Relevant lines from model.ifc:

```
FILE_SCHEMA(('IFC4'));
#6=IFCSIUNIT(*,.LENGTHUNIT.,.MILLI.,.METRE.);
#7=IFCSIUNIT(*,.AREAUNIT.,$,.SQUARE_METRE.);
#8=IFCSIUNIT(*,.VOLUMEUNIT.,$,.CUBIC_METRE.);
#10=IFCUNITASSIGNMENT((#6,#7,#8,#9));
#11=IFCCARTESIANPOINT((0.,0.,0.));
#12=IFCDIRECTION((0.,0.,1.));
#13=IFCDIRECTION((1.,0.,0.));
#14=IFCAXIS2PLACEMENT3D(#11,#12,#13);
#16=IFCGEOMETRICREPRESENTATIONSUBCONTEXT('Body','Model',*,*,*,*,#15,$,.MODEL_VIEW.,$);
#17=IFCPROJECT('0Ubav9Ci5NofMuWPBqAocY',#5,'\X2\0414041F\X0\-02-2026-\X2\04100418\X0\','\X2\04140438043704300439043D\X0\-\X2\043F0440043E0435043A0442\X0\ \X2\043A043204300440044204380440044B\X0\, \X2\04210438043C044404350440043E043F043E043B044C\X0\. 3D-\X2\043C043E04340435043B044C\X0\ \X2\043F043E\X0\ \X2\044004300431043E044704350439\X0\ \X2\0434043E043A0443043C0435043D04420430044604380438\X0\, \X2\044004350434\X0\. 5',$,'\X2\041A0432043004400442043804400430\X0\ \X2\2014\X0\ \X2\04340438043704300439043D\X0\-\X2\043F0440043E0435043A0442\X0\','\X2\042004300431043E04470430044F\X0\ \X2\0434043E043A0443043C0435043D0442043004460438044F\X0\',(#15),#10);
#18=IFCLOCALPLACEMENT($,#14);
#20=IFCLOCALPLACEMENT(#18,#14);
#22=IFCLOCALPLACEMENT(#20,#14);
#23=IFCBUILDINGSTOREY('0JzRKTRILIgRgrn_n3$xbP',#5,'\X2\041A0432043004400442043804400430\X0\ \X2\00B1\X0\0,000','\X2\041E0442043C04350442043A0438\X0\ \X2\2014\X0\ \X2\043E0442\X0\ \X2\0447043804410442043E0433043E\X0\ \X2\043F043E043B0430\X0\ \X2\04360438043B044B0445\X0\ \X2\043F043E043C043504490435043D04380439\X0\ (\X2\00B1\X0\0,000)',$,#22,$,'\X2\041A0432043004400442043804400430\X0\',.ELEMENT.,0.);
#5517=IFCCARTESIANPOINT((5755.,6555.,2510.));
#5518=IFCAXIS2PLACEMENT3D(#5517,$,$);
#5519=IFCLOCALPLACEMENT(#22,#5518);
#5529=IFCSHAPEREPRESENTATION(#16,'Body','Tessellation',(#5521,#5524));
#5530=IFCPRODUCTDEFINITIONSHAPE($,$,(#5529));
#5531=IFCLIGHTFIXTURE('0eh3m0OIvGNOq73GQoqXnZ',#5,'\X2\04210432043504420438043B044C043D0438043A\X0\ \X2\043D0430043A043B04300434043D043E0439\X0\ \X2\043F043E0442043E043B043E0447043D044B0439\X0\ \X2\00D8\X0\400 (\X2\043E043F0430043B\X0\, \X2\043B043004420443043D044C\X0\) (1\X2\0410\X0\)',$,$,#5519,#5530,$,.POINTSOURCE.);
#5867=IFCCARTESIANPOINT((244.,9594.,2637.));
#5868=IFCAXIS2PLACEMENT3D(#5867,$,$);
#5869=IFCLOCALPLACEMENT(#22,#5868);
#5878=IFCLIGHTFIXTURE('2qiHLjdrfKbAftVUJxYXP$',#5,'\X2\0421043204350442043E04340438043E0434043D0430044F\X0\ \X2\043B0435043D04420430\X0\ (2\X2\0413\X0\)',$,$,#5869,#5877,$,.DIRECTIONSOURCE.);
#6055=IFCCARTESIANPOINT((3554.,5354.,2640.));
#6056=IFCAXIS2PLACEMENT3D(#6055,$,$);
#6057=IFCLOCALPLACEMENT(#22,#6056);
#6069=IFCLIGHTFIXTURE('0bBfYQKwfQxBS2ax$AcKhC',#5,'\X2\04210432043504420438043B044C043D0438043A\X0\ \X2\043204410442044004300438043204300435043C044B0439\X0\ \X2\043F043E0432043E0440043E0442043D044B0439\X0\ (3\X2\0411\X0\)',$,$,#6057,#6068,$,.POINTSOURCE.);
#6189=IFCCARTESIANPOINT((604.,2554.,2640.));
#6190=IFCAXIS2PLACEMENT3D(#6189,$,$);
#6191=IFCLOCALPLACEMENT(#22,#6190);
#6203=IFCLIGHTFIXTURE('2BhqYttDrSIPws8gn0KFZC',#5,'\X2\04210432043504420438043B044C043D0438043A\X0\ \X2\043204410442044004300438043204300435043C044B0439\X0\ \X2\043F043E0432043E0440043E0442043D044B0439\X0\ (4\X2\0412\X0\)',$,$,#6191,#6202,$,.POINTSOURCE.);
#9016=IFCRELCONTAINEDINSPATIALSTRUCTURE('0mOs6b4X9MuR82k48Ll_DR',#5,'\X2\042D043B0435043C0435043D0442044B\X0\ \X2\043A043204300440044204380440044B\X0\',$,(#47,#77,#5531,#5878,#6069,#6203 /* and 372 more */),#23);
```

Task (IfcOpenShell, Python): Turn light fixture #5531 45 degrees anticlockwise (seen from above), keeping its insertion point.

```python
import ifcopenshell
import ifcopenshell.api.geometry
import ifcopenshell.util.placement

model = ifcopenshell.open("model.ifc")

item = model.by_id(5531)
matrix = ifcopenshell.util.placement.get_local_placement(item.ObjectPlacement)
matrix = matrix @ ifcopenshell.util.placement.rotation(45, "Z")
ifcopenshell.api.geometry.edit_object_placement(model, product=item, matrix=matrix, is_si=False)

print(ifcopenshell.util.placement.get_local_placement(item.ObjectPlacement).round(3) + 0.0)

model.write("model_rev.ifc")
```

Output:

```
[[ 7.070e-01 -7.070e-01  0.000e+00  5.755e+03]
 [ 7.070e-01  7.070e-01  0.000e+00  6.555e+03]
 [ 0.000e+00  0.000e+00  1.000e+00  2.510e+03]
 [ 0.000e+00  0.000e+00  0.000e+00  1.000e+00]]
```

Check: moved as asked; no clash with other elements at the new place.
